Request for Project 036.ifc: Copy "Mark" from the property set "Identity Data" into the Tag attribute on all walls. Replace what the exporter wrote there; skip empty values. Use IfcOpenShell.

First a look at what the model holds.

```python
import ifcopenshell
import ifcopenshell.util.element

model = ifcopenshell.open("Project 036.ifc")
print(model.schema)
walls = model.by_type("IfcWall")
print(len(walls), "walls")
for e in walls[:8]:
    source = ifcopenshell.util.element.get_pset(e, "Identity Data", "Mark")
    target = e.Tag
    print(e.id(), repr(source), repr(target), sep=" | ")
```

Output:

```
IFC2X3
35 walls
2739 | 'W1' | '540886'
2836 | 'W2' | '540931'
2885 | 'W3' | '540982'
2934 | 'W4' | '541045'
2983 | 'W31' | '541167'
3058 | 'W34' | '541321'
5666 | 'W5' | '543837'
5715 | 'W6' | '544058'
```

```python
import ifcopenshell
import ifcopenshell.util.element

model = ifcopenshell.open("Project 036.ifc")

count = 0
for e in model.by_type("IfcWall"):
    value = ifcopenshell.util.element.get_pset(e, "Identity Data", "Mark")
    current = e.Tag
    if not value or not value.strip() or current == value:
        continue
    e.Tag = value
    count += 1

print(count, "walls updated")

model.write("Project 036_updated.ifc")
```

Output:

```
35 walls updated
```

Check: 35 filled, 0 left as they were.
